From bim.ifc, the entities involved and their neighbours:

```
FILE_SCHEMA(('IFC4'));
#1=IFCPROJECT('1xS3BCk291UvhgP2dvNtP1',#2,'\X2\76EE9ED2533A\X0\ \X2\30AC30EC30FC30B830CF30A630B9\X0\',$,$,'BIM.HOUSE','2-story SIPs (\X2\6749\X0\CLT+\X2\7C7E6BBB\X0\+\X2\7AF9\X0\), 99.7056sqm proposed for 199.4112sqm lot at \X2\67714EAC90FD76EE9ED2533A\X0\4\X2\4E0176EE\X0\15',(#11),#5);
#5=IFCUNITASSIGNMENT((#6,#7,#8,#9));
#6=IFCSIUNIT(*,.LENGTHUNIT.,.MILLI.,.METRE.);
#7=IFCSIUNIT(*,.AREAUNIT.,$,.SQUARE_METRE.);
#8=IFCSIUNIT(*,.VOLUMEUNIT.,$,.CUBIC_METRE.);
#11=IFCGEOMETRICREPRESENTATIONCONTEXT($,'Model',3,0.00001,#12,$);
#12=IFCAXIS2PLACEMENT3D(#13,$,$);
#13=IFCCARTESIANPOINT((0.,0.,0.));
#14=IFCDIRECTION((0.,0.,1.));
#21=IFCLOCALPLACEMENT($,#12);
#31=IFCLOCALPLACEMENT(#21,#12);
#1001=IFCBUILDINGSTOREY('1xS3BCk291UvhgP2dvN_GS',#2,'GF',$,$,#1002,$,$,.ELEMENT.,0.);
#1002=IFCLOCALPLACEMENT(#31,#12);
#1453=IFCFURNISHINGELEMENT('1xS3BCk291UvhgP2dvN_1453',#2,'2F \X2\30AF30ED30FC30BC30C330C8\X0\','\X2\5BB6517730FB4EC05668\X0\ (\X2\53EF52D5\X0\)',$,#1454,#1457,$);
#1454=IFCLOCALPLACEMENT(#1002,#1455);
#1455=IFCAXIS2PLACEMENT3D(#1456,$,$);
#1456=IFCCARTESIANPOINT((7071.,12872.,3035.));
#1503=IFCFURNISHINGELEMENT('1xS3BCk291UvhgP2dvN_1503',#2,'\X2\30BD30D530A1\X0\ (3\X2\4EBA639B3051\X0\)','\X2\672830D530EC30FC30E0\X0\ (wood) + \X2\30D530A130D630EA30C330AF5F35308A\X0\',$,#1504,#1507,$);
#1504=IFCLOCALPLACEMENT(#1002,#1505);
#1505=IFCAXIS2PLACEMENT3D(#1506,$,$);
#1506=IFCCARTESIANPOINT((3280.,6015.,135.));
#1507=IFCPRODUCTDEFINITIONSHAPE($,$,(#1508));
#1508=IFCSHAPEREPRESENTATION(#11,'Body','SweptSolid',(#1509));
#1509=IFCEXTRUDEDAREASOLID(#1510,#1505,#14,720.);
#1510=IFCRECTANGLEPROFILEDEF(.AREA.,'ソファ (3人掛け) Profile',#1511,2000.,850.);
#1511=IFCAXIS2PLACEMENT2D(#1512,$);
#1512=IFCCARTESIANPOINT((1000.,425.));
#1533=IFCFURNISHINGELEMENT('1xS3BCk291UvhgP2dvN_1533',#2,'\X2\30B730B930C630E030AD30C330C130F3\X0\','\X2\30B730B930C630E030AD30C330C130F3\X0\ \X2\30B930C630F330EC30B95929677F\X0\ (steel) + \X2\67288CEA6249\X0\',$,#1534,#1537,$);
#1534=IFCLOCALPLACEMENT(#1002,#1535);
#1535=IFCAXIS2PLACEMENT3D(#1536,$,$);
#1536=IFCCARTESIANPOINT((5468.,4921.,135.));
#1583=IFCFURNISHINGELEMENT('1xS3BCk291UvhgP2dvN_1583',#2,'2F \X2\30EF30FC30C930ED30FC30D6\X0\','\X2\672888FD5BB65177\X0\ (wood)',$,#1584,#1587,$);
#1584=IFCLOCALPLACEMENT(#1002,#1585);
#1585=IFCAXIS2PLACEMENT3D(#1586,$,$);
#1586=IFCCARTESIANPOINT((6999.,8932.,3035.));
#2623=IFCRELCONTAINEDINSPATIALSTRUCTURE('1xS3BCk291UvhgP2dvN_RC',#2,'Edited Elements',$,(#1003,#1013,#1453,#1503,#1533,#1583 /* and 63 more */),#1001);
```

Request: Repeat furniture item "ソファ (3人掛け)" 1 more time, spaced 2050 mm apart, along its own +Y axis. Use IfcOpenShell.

```python
import ifcopenshell
import ifcopenshell.api.geometry
import ifcopenshell.api.root
import ifcopenshell.util.element
import ifcopenshell.util.placement
import ifcopenshell.util.unit

model = ifcopenshell.open("bim.ifc")
unit_scale = ifcopenshell.util.unit.calculate_unit_scale(model)


def reuse_history(source, copy):
    """copy_class also copies each property set's owner history, people and application; keep the originals."""
    for rel in copy.IsDefinedBy:
        if rel.is_a("IfcRelDefinesByProperties") and (history := rel.RelatingPropertyDefinition.OwnerHistory):
            rel.RelatingPropertyDefinition.OwnerHistory = source.OwnerHistory
            ifcopenshell.util.element.remove_deep2(model, history)


source = model.by_id(1503)
base = ifcopenshell.util.placement.get_local_placement(source.ObjectPlacement)
step = base[:3, 1] * 2.05 / unit_scale

for i in range(1, 2):
    copy = ifcopenshell.api.root.copy_class(model, product=source)
    copy.Representation = ifcopenshell.util.element.copy_deep(
        model, source.Representation, exclude=["IfcGeometricRepresentationContext", "IfcRepresentationMap"]
    )
    reuse_history(source, copy)
    matrix = base.copy()
    matrix[:3, 3] += i * step
    print("added at", matrix[:3, 3].round(3) + 0.0)
    ifcopenshell.api.geometry.edit_object_placement(model, product=copy, matrix=matrix, is_si=False)

model.write("bim_updated.ifc")
```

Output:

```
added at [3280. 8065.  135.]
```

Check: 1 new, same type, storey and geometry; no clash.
